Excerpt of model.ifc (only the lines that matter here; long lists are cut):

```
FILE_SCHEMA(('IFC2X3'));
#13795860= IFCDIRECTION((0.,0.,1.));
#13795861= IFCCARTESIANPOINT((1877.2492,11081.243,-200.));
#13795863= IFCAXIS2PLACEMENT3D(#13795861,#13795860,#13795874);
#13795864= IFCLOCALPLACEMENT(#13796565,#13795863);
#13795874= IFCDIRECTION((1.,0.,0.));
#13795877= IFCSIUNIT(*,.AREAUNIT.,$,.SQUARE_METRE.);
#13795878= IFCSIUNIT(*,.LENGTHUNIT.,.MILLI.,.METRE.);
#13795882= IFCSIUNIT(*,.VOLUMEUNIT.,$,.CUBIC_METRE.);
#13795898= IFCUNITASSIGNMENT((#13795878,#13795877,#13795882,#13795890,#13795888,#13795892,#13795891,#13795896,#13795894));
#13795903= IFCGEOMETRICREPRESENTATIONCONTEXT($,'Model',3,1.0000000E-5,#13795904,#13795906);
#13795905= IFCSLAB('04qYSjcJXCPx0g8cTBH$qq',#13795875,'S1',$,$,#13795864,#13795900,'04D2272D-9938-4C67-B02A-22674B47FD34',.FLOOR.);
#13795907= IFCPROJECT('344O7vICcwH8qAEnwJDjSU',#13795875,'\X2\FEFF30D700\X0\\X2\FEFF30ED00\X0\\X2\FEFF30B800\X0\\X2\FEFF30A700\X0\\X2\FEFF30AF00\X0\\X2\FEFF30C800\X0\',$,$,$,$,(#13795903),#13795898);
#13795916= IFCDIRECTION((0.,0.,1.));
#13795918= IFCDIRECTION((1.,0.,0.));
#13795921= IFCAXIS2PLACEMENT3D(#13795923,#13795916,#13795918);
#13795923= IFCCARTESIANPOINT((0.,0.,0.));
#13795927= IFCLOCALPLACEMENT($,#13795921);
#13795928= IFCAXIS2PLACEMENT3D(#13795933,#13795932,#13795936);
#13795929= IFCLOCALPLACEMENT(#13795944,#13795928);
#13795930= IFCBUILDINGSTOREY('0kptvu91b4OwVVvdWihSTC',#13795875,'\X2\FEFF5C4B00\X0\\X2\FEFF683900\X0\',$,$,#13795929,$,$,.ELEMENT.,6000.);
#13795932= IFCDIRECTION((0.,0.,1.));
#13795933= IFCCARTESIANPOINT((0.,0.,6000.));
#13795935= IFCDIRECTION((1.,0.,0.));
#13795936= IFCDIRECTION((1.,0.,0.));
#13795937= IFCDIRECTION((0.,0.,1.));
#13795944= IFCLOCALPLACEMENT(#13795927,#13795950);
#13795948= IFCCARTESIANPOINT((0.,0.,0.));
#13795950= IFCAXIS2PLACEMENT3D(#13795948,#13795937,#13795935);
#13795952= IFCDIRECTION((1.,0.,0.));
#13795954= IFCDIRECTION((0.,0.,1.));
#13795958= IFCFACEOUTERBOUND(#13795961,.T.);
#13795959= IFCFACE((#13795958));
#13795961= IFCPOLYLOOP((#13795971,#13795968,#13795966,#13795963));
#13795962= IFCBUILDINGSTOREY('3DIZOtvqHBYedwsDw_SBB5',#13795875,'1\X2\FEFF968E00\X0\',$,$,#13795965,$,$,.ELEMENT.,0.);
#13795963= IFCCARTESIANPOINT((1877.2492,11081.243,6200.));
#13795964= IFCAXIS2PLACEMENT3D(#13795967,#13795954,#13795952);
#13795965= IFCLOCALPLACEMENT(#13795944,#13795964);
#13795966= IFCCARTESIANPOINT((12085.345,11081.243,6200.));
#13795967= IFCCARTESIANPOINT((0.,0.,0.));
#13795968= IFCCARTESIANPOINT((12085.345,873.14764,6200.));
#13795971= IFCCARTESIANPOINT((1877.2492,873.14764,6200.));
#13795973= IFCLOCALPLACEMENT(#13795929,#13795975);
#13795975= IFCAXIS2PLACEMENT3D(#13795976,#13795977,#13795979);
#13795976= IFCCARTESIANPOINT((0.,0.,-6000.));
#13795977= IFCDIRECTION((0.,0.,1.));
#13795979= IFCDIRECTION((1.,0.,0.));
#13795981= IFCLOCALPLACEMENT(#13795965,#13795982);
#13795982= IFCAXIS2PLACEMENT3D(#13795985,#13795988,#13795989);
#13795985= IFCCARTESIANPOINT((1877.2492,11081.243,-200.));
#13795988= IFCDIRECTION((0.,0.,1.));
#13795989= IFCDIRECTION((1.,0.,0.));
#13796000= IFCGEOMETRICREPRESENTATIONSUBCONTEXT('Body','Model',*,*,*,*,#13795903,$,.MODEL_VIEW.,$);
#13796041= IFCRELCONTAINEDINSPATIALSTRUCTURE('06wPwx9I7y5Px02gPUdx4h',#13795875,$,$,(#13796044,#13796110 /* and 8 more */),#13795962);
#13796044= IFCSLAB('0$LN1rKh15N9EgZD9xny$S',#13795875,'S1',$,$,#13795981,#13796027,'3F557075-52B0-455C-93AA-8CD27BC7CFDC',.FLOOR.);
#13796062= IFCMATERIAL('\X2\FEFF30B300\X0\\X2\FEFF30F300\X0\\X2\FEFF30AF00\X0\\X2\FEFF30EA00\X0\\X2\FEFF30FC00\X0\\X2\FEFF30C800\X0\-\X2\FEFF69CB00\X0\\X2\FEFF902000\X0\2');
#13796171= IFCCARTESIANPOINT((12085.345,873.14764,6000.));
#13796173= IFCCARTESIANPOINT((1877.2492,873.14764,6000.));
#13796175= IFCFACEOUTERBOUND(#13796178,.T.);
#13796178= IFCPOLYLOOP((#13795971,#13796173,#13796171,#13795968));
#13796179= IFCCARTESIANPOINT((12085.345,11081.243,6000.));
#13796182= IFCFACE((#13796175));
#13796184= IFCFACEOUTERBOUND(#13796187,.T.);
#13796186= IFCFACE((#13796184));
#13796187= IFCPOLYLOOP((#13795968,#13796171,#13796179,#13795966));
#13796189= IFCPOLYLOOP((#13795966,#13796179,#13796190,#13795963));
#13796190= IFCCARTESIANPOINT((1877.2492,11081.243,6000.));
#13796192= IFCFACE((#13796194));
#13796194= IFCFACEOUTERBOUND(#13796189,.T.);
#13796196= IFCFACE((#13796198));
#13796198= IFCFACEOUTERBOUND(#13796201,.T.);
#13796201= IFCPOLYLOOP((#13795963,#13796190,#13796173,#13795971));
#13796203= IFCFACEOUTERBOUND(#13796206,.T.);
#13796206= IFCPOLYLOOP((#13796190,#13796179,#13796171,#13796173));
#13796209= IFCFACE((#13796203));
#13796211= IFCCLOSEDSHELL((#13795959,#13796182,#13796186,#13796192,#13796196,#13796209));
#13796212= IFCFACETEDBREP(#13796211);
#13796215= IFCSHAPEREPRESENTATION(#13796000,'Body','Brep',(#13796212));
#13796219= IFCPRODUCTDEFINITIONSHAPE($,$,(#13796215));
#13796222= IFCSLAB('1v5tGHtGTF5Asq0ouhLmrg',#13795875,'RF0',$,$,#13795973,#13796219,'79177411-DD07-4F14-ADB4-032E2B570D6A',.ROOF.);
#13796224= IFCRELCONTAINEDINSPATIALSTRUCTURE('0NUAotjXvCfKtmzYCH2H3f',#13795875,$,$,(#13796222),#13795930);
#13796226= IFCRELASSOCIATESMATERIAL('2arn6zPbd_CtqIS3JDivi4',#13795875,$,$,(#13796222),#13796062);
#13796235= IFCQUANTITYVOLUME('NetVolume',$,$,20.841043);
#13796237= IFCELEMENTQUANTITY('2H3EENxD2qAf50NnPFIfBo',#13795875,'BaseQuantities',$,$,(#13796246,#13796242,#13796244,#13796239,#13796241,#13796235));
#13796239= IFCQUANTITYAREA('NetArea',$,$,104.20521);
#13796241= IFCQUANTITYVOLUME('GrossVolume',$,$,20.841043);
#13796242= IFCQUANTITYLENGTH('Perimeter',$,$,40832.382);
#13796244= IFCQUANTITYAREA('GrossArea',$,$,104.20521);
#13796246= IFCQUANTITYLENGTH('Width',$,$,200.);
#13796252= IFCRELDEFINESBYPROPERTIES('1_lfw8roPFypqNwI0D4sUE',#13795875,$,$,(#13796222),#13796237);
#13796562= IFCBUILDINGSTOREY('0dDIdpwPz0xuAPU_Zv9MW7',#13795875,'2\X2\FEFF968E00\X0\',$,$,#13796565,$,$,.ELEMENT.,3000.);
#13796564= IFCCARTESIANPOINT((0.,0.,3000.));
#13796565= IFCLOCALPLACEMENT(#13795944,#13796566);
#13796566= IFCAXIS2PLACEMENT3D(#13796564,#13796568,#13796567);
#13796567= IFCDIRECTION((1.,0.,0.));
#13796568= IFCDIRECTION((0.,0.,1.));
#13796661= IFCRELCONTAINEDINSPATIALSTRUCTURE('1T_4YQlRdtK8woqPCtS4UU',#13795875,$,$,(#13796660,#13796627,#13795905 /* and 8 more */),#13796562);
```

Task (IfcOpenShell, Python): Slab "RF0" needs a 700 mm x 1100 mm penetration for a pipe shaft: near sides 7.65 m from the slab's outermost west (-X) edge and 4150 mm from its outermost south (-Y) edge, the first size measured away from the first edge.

```python
import numpy as np
import ifcopenshell
import ifcopenshell.api.feature
import ifcopenshell.api.geometry
import ifcopenshell.api.pset
import ifcopenshell.api.root
import ifcopenshell.geom
import ifcopenshell.util.element
import ifcopenshell.util.placement
import ifcopenshell.util.representation
import ifcopenshell.util.shape
import ifcopenshell.util.unit

model = ifcopenshell.open("model.ifc")
unit_scale = ifcopenshell.util.unit.calculate_unit_scale(model)
area_scale = ifcopenshell.util.unit.calculate_unit_scale(model, "AREAUNIT")
volume_scale = ifcopenshell.util.unit.calculate_unit_scale(model, "VOLUMEUNIT")
settings = ifcopenshell.geom.settings()


def volume(element):
    """Net volume in cubic metres, openings subtracted."""
    shape = ifcopenshell.geom.create_shape(settings, element)
    return ifcopenshell.util.shape.get_volume(shape.geometry)


slab = model.by_id(13796222)
before = volume(slab)

# Extent in the slab's own axes, in metres. The edges named are its -X and -Y sides.
slab_shape = ifcopenshell.geom.create_shape(settings, slab)
vertices = ifcopenshell.util.shape.get_vertices(slab_shape.geometry)
x_min, y_min, bottom = vertices.min(axis=0)
top = vertices[:, 2].max()

opening = ifcopenshell.api.root.create_entity(model, ifc_class="IfcOpeningElement", name="Pipe shaft opening")
context = ifcopenshell.util.representation.get_context(model, "Model", "Body", "MODEL_VIEW")
width, depth = 0.7, 1.1
outline = [(0.0, 0.0), (width, 0.0), (width, depth), (0.0, depth), (0.0, 0.0)]
# Overshoot both faces by 50 mm so the cut is clean.
shape = ifcopenshell.api.geometry.add_slab_representation(
    model, context=context, depth=top - bottom + 0.1, polyline=outline
)
ifcopenshell.api.geometry.assign_representation(model, product=opening, representation=shape)

matrix = ifcopenshell.util.placement.get_local_placement(slab.ObjectPlacement)
matrix[:, 3] = matrix @ np.append(np.array([x_min + 7.65, y_min + 4.15, bottom - 0.05]) / unit_scale, 1.0)
ifcopenshell.api.geometry.edit_object_placement(model, product=opening, matrix=matrix, is_si=False)
ifcopenshell.api.feature.add_feature(model, feature=opening, element=slab)

after = volume(slab)

# Update the slab's stored quantities.
qto = model.by_id(ifcopenshell.util.element.get_pset(slab, "BaseQuantities", should_inherit=False)["id"])
ifcopenshell.api.pset.edit_qto(model, qto=qto, properties={
    "NetArea": after / (top - bottom) / area_scale,
    "NetVolume": after / volume_scale,
})

print(f"slab volume {before:.3f} -> {after:.3f} m3")

model.write("model_edited.ifc")
```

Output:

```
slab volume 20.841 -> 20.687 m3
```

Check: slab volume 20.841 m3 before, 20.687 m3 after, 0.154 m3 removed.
